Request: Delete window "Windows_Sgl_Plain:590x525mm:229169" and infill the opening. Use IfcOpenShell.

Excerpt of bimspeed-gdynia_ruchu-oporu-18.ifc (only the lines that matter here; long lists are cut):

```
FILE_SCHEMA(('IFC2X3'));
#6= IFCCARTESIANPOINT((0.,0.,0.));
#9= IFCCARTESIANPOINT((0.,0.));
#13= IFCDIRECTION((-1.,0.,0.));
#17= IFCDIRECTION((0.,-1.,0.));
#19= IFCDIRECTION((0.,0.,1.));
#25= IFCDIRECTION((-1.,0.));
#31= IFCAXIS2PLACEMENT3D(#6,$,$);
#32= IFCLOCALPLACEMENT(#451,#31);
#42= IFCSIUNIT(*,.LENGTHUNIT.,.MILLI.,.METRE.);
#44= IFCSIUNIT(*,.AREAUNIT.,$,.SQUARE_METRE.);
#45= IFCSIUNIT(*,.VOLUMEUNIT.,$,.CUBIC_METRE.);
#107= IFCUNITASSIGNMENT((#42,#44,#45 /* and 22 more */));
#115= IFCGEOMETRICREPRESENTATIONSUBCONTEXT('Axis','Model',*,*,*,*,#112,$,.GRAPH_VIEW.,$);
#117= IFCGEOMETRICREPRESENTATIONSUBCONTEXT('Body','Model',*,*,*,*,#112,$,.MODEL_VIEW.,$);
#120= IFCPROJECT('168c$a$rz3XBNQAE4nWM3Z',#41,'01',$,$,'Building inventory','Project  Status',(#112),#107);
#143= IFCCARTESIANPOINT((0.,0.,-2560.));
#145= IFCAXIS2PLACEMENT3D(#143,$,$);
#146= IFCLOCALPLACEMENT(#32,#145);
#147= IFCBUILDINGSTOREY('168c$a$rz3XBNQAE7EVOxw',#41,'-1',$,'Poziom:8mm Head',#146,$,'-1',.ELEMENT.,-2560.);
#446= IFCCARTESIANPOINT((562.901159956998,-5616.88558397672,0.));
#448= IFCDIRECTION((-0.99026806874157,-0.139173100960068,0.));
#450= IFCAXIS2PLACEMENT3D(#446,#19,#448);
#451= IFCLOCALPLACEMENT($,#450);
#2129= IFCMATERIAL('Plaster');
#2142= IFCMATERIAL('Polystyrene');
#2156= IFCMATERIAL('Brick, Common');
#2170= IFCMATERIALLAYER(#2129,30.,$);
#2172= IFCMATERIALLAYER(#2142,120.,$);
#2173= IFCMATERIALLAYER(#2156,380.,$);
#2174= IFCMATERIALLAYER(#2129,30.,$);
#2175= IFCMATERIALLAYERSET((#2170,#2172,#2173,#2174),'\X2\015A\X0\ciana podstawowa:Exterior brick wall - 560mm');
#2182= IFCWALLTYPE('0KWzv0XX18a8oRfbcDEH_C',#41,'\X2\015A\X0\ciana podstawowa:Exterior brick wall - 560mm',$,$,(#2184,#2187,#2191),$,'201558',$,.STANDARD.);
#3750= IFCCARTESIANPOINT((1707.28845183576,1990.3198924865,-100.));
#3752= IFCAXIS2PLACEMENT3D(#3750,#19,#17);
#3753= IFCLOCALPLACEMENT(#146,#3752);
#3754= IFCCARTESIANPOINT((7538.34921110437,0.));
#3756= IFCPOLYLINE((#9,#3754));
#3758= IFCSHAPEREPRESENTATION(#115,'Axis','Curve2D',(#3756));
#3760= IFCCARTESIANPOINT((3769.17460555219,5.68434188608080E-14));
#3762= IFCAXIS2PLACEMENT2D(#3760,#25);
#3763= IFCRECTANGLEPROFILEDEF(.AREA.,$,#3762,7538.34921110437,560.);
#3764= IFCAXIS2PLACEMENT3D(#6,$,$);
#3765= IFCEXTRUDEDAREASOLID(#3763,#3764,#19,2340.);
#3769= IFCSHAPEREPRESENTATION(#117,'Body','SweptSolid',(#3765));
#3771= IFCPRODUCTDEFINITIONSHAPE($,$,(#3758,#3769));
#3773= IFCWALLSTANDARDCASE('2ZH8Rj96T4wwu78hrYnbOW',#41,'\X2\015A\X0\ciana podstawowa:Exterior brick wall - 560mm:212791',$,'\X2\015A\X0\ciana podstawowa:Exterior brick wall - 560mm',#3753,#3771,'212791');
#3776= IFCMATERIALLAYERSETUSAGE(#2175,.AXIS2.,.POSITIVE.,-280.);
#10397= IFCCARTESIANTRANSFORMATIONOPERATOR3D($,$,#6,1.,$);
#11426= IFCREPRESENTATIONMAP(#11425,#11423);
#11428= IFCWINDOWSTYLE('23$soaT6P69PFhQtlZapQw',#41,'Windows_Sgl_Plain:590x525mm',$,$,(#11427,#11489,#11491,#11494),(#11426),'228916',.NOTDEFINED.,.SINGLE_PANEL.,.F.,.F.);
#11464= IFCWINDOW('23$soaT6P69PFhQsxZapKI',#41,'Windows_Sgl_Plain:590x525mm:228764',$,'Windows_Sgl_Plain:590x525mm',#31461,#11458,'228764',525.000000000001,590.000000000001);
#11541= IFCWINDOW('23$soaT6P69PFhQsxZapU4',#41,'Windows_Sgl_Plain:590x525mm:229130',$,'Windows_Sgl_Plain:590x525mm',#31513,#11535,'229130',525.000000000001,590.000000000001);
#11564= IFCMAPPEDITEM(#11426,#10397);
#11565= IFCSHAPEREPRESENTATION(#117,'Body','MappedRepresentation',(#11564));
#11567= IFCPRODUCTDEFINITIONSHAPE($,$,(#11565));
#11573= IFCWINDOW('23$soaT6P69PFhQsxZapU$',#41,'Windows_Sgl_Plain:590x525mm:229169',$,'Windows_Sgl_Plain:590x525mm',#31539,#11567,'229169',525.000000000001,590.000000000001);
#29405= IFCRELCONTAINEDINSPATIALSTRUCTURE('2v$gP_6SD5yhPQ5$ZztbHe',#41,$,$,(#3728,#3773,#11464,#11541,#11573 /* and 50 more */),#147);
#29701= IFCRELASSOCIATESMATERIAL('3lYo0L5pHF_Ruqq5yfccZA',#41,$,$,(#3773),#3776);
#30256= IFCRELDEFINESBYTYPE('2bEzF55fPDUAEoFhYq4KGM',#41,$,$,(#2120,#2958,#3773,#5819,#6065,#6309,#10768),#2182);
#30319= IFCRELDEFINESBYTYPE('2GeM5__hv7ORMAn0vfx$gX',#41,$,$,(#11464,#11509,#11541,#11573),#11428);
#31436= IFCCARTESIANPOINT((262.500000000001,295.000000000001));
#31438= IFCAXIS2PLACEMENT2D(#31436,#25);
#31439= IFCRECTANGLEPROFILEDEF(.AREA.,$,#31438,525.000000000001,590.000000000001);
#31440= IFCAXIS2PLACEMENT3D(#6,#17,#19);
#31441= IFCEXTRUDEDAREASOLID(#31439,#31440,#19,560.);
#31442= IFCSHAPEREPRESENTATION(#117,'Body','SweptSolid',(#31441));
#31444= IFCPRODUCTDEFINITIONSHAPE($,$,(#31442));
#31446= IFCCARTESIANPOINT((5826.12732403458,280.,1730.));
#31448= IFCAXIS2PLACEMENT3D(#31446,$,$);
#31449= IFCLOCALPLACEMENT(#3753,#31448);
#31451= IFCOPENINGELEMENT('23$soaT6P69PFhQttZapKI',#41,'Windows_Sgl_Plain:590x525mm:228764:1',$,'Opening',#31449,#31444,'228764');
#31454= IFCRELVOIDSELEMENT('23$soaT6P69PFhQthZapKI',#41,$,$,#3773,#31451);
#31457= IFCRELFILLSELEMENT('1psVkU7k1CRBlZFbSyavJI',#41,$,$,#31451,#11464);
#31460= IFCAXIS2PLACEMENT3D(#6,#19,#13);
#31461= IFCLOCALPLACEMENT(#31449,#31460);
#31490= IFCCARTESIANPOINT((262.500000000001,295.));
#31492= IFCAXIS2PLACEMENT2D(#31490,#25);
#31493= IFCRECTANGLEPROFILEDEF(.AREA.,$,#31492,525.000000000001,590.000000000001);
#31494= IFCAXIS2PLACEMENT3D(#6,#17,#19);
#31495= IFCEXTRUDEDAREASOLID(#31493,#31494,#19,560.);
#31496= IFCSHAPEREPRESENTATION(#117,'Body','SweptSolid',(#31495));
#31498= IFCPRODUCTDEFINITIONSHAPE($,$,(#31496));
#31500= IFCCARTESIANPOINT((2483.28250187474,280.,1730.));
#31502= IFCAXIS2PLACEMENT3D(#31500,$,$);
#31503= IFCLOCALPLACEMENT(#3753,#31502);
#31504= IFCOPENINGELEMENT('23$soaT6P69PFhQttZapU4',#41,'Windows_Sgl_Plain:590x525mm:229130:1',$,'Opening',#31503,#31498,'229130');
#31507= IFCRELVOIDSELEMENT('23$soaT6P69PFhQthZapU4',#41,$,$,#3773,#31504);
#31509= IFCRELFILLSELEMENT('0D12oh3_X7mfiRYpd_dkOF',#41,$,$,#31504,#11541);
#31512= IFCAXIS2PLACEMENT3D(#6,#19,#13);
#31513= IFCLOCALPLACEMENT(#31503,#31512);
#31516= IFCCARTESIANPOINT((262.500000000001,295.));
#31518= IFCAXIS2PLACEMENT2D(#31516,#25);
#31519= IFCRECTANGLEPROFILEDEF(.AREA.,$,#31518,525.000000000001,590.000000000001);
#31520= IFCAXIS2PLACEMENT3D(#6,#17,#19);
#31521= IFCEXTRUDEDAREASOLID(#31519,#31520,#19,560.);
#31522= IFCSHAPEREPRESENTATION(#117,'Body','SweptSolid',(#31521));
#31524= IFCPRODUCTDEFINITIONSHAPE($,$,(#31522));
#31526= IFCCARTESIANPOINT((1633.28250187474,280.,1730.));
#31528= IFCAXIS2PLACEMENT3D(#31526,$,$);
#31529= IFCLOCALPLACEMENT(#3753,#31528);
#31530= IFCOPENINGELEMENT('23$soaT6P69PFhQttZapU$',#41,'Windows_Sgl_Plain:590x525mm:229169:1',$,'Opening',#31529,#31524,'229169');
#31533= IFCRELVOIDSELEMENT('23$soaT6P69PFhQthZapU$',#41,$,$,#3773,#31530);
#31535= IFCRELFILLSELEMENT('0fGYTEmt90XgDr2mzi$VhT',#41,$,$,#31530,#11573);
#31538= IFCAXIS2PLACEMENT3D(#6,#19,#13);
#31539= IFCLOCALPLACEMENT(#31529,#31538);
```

```python
import ifcopenshell
import ifcopenshell.api.feature
import ifcopenshell.api.root
import ifcopenshell.geom
import ifcopenshell.util.shape

model = ifcopenshell.open("bimspeed-gdynia_ruchu-oporu-18.ifc")
settings = ifcopenshell.geom.settings()


def volume(element):
    """Net volume in cubic metres, openings subtracted."""
    shape = ifcopenshell.geom.create_shape(settings, element)
    return ifcopenshell.util.shape.get_volume(shape.geometry)


window = model.by_guid("23$soaT6P69PFhQsxZapU$")
opening = window.FillsVoids[0].RelatingOpeningElement
wall = opening.VoidsElements[0].RelatingBuildingElement
before = volume(wall)

ifcopenshell.api.root.remove_product(model, product=window)
ifcopenshell.api.feature.remove_feature(model, feature=opening)

after = volume(wall)

print(f"wall volume {before:.3f} -> {after:.3f} m3")

model.write("bimspeed-gdynia_ruchu-oporu-18_edited.ifc")
```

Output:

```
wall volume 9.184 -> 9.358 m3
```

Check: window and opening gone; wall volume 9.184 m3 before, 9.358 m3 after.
